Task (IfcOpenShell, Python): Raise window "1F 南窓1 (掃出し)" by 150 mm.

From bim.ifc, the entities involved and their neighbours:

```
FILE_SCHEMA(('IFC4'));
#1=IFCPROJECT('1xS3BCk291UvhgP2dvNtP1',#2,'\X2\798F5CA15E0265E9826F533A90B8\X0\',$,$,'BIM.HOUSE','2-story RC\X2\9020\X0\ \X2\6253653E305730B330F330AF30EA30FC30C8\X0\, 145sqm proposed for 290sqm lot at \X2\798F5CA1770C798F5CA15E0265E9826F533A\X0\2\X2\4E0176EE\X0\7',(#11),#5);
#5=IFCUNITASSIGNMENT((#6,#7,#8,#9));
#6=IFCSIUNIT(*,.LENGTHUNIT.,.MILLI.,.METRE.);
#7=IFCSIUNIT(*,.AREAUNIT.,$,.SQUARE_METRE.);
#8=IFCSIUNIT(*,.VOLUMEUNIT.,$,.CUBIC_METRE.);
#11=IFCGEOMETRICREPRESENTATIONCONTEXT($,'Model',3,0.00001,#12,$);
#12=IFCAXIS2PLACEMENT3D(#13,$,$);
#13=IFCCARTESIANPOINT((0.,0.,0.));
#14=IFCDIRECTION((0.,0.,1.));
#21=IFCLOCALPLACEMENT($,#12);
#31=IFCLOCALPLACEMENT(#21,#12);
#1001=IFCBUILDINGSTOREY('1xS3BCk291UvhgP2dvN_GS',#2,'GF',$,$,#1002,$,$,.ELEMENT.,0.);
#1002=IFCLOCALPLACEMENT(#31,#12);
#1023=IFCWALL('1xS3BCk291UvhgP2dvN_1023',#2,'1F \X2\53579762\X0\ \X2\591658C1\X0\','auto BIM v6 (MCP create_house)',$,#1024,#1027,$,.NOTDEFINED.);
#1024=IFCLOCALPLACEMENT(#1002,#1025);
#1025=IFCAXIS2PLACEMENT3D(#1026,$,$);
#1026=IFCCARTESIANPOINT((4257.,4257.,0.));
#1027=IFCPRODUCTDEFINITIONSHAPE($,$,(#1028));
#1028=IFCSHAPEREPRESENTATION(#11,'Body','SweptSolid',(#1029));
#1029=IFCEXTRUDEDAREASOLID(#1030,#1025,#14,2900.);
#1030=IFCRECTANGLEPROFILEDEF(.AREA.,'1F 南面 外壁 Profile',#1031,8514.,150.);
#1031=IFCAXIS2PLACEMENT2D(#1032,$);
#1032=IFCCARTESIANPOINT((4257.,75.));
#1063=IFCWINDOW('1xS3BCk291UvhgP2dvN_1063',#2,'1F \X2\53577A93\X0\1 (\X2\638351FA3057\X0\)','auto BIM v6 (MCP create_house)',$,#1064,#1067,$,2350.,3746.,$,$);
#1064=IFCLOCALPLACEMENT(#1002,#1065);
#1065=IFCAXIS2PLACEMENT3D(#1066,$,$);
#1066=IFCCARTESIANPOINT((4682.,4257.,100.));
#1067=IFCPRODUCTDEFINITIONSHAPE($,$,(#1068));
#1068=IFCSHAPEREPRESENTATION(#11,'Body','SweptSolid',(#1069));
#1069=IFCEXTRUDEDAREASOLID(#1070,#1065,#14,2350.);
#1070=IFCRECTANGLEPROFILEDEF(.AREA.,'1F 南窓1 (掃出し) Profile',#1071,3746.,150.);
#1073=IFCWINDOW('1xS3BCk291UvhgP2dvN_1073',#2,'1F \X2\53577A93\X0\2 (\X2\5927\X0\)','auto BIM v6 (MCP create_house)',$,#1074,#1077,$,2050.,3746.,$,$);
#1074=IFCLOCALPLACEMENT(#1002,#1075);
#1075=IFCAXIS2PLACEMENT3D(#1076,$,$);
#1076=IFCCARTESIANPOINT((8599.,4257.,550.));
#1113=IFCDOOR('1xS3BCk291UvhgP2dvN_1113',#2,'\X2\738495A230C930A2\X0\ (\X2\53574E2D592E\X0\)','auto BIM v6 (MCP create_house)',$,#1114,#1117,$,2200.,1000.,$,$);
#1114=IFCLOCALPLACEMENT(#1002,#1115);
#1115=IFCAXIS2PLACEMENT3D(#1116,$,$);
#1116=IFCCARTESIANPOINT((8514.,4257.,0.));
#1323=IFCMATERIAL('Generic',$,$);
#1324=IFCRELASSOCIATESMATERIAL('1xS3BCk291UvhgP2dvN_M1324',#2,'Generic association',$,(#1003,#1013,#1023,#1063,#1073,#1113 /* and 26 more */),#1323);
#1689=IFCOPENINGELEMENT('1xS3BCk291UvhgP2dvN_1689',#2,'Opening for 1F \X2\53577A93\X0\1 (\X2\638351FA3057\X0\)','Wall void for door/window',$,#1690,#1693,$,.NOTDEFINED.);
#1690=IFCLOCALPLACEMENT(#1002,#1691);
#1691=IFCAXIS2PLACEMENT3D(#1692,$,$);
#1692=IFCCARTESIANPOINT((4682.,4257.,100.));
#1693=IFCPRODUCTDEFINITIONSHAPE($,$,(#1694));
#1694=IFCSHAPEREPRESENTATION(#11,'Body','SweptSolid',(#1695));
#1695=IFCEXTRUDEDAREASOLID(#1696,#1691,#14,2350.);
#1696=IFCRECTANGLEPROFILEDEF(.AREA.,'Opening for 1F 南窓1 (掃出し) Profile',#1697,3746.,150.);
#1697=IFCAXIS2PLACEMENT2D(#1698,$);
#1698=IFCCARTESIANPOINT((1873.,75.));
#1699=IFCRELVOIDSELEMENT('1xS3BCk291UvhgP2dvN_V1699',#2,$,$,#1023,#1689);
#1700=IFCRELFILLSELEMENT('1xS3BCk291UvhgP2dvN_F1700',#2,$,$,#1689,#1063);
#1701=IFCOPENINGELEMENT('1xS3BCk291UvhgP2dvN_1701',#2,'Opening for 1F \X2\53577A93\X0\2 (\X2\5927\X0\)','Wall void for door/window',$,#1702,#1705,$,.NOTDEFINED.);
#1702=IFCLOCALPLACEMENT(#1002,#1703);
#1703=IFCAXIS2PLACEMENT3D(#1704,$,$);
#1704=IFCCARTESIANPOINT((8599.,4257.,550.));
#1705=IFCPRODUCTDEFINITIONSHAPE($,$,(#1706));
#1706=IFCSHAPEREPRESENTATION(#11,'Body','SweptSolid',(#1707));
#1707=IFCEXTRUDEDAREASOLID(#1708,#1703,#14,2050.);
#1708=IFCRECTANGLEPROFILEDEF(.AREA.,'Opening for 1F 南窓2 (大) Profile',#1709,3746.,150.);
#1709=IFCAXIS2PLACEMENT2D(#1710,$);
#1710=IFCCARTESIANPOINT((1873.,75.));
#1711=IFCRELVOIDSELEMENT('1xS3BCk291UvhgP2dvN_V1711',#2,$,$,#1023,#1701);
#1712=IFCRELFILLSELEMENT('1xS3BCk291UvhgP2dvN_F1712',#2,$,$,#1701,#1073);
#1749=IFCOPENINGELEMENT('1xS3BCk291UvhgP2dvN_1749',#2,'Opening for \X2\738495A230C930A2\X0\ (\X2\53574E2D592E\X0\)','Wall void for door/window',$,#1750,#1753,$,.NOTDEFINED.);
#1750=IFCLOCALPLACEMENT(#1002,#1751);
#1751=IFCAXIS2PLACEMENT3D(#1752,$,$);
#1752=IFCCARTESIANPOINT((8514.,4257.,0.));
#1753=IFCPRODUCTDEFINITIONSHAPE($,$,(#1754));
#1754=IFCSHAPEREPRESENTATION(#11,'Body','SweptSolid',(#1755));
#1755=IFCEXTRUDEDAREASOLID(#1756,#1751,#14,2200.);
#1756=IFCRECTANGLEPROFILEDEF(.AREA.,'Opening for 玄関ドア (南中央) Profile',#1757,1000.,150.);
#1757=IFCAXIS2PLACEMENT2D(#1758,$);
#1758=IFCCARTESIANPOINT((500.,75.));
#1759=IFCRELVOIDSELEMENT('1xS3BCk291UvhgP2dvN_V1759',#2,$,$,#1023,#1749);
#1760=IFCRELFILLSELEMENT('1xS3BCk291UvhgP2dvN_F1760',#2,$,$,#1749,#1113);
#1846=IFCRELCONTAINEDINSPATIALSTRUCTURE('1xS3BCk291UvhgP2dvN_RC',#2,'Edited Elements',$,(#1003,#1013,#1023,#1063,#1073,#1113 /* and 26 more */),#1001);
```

```python
import numpy as np
import ifcopenshell
import ifcopenshell.api.geometry
import ifcopenshell.util.placement
import ifcopenshell.util.unit

model = ifcopenshell.open("bim.ifc")
unit_scale = ifcopenshell.util.unit.calculate_unit_scale(model)

window = model.by_id(1063)
opening = window.FillsVoids[0].RelatingOpeningElement
dz = 150.0

shift = np.array([0.0, 0.0, dz])
# The window is not placed relative to its opening, so move both.
for product in (opening, window):
    matrix = ifcopenshell.util.placement.get_local_placement(product.ObjectPlacement)
    matrix[:3, 3] += shift
    ifcopenshell.api.geometry.edit_object_placement(model, product=product, matrix=matrix, is_si=False)

print(f"moved by {dz * unit_scale:+.3f} m")

model.write("bim_updated.ifc")
```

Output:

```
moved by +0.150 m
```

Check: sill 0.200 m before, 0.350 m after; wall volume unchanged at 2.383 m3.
